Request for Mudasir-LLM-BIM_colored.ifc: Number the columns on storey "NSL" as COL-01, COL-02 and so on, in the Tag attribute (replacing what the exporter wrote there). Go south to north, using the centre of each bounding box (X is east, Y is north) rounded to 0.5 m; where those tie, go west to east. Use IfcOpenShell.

First a look at what the model holds.

```python
import ifcopenshell
import ifcopenshell.util.element
import ifcopenshell.util.placement

model = ifcopenshell.open("Mudasir-LLM-BIM_colored.ifc")
print(model.schema)
storey = next(s for s in model.by_type("IfcBuildingStorey") if s.Name == "NSL")
columns = [e for e in ifcopenshell.util.element.get_decomposition(storey) if e.is_a("IfcColumn")]
for e in sorted(columns, key=lambda e: e.id()):
    origin = ifcopenshell.util.placement.get_local_placement(e.ObjectPlacement)[:3, 3]
    print(e.id(), e.Tag, e.Name, origin.round(2) + 0.0, sep=" | ")
```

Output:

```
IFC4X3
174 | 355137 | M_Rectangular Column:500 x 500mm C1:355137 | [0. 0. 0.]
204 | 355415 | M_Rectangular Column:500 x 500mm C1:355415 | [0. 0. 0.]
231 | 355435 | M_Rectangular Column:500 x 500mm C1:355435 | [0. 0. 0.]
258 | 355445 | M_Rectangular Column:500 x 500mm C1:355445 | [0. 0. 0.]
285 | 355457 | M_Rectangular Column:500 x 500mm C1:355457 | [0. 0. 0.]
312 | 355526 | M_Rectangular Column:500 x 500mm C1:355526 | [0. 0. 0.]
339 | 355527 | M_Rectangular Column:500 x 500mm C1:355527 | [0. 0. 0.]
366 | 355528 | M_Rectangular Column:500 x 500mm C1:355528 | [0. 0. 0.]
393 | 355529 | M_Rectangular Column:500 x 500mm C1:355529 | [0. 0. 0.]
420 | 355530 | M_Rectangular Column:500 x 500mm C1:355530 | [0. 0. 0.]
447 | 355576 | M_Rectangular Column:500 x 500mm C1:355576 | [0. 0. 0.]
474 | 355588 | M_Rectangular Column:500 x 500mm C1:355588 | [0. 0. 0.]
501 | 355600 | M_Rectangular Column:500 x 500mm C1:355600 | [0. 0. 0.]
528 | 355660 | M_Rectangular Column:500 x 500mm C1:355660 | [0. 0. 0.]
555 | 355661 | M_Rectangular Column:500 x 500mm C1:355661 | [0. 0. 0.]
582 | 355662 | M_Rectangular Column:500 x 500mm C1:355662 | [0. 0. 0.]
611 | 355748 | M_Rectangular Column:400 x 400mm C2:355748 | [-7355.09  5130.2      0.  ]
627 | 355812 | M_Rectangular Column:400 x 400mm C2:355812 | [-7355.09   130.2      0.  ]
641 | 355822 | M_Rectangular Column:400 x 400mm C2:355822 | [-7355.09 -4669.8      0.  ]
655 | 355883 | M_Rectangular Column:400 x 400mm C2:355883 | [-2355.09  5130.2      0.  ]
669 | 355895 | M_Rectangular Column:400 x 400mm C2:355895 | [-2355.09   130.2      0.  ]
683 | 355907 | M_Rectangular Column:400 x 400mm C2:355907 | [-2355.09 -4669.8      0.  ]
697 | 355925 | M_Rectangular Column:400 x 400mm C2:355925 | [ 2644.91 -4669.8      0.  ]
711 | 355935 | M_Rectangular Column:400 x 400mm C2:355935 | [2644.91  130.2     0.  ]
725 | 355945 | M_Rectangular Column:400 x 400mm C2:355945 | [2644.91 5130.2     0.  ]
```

```python
import ifcopenshell
import ifcopenshell.geom
import ifcopenshell.util.element
import ifcopenshell.util.shape

model = ifcopenshell.open("Mudasir-LLM-BIM_colored.ifc")
settings = ifcopenshell.geom.settings()
settings.set("use-world-coords", True)


def centre(element):
    shape = ifcopenshell.geom.create_shape(settings, element)
    return ifcopenshell.util.shape.get_bbox_centroid(shape.geometry)


storey = next(s for s in model.by_type("IfcBuildingStorey") if s.Name == "NSL")
columns = [e for e in ifcopenshell.util.element.get_decomposition(storey) if e.is_a("IfcColumn")]

# Insertion points can sit at a corner or the storey origin, so sort by the geometry (in metres).
centres = {e: centre(e) for e in columns}
columns.sort(key=lambda e: (round(centres[e][1] / 0.5), centres[e][0]))

for i, e in enumerate(columns, start=1):
    number = f"COL-{i:02d}"
    e.Tag = number
    print(e.id(), number)

model.write("Mudasir-LLM-BIM_colored_updated.ifc")
```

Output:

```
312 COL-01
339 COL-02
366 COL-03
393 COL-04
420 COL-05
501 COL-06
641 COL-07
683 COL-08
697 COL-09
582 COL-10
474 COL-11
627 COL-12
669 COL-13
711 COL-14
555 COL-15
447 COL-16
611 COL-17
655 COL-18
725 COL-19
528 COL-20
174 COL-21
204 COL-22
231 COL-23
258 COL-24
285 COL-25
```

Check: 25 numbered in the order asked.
